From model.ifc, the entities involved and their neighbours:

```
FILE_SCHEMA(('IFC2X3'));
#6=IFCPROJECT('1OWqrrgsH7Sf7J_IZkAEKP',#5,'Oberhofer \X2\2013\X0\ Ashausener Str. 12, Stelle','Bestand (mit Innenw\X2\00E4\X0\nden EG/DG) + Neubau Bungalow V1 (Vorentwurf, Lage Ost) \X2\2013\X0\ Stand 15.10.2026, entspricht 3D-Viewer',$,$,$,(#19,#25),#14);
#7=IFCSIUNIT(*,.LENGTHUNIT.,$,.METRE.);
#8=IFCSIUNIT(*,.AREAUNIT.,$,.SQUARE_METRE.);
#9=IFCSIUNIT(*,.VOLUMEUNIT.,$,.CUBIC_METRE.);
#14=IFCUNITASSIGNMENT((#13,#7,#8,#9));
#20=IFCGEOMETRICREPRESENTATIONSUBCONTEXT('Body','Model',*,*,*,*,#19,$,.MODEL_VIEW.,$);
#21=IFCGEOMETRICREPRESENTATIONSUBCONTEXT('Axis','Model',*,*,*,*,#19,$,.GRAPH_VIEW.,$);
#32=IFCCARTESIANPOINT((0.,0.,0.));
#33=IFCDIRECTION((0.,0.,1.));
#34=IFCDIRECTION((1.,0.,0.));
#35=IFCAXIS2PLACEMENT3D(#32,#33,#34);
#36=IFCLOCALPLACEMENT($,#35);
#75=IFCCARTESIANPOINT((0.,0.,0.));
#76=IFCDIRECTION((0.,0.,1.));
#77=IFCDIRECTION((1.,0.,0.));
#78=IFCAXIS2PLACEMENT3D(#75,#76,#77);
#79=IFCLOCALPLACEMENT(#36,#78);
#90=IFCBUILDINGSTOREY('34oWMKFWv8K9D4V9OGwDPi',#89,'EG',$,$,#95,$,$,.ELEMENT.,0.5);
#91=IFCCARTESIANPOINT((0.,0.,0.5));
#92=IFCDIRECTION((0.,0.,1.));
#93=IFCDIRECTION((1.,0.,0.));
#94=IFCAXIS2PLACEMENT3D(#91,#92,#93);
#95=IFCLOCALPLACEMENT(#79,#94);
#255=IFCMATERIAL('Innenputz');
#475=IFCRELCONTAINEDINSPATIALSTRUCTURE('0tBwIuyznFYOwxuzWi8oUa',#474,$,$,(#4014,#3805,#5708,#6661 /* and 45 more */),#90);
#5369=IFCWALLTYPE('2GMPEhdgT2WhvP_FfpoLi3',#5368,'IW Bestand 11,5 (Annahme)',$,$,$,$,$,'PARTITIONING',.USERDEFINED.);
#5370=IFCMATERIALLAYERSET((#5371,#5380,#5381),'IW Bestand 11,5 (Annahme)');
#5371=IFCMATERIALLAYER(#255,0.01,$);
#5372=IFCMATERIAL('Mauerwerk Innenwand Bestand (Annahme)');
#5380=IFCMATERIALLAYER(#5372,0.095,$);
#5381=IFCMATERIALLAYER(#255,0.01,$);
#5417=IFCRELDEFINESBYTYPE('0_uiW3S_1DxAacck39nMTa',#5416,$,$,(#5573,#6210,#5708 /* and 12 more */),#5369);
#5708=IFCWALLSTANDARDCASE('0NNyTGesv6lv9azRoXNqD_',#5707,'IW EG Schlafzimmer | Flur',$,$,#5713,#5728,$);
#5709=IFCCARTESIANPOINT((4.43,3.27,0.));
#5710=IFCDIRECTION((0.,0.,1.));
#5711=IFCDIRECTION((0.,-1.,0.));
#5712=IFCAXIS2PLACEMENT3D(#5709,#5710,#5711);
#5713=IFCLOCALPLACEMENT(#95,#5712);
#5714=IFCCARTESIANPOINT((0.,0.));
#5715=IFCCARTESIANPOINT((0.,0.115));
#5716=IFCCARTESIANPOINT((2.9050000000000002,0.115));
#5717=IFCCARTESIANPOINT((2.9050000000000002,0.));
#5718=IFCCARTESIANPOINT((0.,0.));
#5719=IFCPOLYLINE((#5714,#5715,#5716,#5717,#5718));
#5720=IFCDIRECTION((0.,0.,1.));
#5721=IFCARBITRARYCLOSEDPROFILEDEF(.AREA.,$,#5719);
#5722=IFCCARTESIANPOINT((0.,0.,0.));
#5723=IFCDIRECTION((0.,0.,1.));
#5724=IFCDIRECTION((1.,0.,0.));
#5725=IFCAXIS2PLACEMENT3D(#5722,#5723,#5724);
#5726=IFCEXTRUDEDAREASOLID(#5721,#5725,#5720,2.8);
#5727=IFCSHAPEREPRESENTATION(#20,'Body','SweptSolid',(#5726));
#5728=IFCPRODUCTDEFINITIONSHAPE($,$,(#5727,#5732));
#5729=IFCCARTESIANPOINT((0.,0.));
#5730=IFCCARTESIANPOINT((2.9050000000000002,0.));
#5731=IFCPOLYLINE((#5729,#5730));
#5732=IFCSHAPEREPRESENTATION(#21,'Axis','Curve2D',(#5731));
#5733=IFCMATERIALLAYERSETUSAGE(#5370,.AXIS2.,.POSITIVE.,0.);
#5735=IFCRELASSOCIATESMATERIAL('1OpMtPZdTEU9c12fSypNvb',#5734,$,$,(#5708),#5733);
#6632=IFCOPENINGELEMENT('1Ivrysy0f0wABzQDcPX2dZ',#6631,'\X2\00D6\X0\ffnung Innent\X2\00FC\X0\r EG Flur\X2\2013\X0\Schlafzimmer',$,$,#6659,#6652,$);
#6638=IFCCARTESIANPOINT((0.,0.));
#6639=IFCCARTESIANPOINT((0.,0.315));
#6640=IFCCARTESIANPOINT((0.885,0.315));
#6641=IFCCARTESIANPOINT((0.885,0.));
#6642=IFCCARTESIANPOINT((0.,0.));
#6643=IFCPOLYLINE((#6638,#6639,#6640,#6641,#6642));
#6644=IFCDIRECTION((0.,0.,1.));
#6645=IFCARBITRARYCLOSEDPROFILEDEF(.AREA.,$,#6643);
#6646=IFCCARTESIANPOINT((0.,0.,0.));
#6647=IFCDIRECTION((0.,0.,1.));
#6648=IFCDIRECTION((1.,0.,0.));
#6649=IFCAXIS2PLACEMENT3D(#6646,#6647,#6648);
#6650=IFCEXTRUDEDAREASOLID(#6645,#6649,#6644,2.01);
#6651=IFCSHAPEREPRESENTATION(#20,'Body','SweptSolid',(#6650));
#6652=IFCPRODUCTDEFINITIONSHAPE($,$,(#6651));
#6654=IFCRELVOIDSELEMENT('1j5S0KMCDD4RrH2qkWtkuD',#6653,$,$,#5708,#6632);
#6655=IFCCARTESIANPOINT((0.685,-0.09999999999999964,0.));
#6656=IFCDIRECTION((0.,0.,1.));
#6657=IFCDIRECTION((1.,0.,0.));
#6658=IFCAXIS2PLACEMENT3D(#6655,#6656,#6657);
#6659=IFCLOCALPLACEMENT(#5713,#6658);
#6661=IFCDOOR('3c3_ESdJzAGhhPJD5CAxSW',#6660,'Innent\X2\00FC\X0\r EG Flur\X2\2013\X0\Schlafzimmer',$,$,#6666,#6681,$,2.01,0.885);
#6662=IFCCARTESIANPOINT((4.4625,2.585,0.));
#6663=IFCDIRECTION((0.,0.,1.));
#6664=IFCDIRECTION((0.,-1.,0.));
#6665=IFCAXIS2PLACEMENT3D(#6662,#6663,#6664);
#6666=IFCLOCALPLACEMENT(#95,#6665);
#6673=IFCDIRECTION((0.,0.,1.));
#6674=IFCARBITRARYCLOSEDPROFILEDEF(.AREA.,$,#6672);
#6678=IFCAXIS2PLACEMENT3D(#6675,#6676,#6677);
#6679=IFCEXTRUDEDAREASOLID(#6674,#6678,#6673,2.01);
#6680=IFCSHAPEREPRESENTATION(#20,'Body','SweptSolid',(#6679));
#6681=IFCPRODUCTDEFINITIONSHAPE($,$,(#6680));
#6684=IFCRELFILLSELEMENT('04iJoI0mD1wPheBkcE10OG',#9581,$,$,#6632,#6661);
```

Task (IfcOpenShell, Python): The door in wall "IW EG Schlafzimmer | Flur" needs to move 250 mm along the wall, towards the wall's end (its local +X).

```python
import ifcopenshell
import ifcopenshell.api.geometry
import ifcopenshell.util.placement
import ifcopenshell.util.unit

model = ifcopenshell.open("model.ifc")
unit_scale = ifcopenshell.util.unit.calculate_unit_scale(model)

door = model.by_id(6661)
opening = door.FillsVoids[0].RelatingOpeningElement
wall = opening.VoidsElements[0].RelatingBuildingElement

wall_matrix = ifcopenshell.util.placement.get_local_placement(wall.ObjectPlacement)
shift = wall_matrix[:3, 0] * 0.25 / unit_scale
before = ifcopenshell.util.placement.get_local_placement(door.ObjectPlacement)[:3, 3].copy()

# The door is not placed relative to its opening, so move both.
for product in (opening, door):
    matrix = ifcopenshell.util.placement.get_local_placement(product.ObjectPlacement)
    matrix[:3, 3] += shift
    ifcopenshell.api.geometry.edit_object_placement(model, product=product, matrix=matrix, is_si=False)

after = ifcopenshell.util.placement.get_local_placement(door.ObjectPlacement)[:3, 3]
print("door moved by", (after - before).round(3) + 0.0)

model.write("model_rev.ifc")
```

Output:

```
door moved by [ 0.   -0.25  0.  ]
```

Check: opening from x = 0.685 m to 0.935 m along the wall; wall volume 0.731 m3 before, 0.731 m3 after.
